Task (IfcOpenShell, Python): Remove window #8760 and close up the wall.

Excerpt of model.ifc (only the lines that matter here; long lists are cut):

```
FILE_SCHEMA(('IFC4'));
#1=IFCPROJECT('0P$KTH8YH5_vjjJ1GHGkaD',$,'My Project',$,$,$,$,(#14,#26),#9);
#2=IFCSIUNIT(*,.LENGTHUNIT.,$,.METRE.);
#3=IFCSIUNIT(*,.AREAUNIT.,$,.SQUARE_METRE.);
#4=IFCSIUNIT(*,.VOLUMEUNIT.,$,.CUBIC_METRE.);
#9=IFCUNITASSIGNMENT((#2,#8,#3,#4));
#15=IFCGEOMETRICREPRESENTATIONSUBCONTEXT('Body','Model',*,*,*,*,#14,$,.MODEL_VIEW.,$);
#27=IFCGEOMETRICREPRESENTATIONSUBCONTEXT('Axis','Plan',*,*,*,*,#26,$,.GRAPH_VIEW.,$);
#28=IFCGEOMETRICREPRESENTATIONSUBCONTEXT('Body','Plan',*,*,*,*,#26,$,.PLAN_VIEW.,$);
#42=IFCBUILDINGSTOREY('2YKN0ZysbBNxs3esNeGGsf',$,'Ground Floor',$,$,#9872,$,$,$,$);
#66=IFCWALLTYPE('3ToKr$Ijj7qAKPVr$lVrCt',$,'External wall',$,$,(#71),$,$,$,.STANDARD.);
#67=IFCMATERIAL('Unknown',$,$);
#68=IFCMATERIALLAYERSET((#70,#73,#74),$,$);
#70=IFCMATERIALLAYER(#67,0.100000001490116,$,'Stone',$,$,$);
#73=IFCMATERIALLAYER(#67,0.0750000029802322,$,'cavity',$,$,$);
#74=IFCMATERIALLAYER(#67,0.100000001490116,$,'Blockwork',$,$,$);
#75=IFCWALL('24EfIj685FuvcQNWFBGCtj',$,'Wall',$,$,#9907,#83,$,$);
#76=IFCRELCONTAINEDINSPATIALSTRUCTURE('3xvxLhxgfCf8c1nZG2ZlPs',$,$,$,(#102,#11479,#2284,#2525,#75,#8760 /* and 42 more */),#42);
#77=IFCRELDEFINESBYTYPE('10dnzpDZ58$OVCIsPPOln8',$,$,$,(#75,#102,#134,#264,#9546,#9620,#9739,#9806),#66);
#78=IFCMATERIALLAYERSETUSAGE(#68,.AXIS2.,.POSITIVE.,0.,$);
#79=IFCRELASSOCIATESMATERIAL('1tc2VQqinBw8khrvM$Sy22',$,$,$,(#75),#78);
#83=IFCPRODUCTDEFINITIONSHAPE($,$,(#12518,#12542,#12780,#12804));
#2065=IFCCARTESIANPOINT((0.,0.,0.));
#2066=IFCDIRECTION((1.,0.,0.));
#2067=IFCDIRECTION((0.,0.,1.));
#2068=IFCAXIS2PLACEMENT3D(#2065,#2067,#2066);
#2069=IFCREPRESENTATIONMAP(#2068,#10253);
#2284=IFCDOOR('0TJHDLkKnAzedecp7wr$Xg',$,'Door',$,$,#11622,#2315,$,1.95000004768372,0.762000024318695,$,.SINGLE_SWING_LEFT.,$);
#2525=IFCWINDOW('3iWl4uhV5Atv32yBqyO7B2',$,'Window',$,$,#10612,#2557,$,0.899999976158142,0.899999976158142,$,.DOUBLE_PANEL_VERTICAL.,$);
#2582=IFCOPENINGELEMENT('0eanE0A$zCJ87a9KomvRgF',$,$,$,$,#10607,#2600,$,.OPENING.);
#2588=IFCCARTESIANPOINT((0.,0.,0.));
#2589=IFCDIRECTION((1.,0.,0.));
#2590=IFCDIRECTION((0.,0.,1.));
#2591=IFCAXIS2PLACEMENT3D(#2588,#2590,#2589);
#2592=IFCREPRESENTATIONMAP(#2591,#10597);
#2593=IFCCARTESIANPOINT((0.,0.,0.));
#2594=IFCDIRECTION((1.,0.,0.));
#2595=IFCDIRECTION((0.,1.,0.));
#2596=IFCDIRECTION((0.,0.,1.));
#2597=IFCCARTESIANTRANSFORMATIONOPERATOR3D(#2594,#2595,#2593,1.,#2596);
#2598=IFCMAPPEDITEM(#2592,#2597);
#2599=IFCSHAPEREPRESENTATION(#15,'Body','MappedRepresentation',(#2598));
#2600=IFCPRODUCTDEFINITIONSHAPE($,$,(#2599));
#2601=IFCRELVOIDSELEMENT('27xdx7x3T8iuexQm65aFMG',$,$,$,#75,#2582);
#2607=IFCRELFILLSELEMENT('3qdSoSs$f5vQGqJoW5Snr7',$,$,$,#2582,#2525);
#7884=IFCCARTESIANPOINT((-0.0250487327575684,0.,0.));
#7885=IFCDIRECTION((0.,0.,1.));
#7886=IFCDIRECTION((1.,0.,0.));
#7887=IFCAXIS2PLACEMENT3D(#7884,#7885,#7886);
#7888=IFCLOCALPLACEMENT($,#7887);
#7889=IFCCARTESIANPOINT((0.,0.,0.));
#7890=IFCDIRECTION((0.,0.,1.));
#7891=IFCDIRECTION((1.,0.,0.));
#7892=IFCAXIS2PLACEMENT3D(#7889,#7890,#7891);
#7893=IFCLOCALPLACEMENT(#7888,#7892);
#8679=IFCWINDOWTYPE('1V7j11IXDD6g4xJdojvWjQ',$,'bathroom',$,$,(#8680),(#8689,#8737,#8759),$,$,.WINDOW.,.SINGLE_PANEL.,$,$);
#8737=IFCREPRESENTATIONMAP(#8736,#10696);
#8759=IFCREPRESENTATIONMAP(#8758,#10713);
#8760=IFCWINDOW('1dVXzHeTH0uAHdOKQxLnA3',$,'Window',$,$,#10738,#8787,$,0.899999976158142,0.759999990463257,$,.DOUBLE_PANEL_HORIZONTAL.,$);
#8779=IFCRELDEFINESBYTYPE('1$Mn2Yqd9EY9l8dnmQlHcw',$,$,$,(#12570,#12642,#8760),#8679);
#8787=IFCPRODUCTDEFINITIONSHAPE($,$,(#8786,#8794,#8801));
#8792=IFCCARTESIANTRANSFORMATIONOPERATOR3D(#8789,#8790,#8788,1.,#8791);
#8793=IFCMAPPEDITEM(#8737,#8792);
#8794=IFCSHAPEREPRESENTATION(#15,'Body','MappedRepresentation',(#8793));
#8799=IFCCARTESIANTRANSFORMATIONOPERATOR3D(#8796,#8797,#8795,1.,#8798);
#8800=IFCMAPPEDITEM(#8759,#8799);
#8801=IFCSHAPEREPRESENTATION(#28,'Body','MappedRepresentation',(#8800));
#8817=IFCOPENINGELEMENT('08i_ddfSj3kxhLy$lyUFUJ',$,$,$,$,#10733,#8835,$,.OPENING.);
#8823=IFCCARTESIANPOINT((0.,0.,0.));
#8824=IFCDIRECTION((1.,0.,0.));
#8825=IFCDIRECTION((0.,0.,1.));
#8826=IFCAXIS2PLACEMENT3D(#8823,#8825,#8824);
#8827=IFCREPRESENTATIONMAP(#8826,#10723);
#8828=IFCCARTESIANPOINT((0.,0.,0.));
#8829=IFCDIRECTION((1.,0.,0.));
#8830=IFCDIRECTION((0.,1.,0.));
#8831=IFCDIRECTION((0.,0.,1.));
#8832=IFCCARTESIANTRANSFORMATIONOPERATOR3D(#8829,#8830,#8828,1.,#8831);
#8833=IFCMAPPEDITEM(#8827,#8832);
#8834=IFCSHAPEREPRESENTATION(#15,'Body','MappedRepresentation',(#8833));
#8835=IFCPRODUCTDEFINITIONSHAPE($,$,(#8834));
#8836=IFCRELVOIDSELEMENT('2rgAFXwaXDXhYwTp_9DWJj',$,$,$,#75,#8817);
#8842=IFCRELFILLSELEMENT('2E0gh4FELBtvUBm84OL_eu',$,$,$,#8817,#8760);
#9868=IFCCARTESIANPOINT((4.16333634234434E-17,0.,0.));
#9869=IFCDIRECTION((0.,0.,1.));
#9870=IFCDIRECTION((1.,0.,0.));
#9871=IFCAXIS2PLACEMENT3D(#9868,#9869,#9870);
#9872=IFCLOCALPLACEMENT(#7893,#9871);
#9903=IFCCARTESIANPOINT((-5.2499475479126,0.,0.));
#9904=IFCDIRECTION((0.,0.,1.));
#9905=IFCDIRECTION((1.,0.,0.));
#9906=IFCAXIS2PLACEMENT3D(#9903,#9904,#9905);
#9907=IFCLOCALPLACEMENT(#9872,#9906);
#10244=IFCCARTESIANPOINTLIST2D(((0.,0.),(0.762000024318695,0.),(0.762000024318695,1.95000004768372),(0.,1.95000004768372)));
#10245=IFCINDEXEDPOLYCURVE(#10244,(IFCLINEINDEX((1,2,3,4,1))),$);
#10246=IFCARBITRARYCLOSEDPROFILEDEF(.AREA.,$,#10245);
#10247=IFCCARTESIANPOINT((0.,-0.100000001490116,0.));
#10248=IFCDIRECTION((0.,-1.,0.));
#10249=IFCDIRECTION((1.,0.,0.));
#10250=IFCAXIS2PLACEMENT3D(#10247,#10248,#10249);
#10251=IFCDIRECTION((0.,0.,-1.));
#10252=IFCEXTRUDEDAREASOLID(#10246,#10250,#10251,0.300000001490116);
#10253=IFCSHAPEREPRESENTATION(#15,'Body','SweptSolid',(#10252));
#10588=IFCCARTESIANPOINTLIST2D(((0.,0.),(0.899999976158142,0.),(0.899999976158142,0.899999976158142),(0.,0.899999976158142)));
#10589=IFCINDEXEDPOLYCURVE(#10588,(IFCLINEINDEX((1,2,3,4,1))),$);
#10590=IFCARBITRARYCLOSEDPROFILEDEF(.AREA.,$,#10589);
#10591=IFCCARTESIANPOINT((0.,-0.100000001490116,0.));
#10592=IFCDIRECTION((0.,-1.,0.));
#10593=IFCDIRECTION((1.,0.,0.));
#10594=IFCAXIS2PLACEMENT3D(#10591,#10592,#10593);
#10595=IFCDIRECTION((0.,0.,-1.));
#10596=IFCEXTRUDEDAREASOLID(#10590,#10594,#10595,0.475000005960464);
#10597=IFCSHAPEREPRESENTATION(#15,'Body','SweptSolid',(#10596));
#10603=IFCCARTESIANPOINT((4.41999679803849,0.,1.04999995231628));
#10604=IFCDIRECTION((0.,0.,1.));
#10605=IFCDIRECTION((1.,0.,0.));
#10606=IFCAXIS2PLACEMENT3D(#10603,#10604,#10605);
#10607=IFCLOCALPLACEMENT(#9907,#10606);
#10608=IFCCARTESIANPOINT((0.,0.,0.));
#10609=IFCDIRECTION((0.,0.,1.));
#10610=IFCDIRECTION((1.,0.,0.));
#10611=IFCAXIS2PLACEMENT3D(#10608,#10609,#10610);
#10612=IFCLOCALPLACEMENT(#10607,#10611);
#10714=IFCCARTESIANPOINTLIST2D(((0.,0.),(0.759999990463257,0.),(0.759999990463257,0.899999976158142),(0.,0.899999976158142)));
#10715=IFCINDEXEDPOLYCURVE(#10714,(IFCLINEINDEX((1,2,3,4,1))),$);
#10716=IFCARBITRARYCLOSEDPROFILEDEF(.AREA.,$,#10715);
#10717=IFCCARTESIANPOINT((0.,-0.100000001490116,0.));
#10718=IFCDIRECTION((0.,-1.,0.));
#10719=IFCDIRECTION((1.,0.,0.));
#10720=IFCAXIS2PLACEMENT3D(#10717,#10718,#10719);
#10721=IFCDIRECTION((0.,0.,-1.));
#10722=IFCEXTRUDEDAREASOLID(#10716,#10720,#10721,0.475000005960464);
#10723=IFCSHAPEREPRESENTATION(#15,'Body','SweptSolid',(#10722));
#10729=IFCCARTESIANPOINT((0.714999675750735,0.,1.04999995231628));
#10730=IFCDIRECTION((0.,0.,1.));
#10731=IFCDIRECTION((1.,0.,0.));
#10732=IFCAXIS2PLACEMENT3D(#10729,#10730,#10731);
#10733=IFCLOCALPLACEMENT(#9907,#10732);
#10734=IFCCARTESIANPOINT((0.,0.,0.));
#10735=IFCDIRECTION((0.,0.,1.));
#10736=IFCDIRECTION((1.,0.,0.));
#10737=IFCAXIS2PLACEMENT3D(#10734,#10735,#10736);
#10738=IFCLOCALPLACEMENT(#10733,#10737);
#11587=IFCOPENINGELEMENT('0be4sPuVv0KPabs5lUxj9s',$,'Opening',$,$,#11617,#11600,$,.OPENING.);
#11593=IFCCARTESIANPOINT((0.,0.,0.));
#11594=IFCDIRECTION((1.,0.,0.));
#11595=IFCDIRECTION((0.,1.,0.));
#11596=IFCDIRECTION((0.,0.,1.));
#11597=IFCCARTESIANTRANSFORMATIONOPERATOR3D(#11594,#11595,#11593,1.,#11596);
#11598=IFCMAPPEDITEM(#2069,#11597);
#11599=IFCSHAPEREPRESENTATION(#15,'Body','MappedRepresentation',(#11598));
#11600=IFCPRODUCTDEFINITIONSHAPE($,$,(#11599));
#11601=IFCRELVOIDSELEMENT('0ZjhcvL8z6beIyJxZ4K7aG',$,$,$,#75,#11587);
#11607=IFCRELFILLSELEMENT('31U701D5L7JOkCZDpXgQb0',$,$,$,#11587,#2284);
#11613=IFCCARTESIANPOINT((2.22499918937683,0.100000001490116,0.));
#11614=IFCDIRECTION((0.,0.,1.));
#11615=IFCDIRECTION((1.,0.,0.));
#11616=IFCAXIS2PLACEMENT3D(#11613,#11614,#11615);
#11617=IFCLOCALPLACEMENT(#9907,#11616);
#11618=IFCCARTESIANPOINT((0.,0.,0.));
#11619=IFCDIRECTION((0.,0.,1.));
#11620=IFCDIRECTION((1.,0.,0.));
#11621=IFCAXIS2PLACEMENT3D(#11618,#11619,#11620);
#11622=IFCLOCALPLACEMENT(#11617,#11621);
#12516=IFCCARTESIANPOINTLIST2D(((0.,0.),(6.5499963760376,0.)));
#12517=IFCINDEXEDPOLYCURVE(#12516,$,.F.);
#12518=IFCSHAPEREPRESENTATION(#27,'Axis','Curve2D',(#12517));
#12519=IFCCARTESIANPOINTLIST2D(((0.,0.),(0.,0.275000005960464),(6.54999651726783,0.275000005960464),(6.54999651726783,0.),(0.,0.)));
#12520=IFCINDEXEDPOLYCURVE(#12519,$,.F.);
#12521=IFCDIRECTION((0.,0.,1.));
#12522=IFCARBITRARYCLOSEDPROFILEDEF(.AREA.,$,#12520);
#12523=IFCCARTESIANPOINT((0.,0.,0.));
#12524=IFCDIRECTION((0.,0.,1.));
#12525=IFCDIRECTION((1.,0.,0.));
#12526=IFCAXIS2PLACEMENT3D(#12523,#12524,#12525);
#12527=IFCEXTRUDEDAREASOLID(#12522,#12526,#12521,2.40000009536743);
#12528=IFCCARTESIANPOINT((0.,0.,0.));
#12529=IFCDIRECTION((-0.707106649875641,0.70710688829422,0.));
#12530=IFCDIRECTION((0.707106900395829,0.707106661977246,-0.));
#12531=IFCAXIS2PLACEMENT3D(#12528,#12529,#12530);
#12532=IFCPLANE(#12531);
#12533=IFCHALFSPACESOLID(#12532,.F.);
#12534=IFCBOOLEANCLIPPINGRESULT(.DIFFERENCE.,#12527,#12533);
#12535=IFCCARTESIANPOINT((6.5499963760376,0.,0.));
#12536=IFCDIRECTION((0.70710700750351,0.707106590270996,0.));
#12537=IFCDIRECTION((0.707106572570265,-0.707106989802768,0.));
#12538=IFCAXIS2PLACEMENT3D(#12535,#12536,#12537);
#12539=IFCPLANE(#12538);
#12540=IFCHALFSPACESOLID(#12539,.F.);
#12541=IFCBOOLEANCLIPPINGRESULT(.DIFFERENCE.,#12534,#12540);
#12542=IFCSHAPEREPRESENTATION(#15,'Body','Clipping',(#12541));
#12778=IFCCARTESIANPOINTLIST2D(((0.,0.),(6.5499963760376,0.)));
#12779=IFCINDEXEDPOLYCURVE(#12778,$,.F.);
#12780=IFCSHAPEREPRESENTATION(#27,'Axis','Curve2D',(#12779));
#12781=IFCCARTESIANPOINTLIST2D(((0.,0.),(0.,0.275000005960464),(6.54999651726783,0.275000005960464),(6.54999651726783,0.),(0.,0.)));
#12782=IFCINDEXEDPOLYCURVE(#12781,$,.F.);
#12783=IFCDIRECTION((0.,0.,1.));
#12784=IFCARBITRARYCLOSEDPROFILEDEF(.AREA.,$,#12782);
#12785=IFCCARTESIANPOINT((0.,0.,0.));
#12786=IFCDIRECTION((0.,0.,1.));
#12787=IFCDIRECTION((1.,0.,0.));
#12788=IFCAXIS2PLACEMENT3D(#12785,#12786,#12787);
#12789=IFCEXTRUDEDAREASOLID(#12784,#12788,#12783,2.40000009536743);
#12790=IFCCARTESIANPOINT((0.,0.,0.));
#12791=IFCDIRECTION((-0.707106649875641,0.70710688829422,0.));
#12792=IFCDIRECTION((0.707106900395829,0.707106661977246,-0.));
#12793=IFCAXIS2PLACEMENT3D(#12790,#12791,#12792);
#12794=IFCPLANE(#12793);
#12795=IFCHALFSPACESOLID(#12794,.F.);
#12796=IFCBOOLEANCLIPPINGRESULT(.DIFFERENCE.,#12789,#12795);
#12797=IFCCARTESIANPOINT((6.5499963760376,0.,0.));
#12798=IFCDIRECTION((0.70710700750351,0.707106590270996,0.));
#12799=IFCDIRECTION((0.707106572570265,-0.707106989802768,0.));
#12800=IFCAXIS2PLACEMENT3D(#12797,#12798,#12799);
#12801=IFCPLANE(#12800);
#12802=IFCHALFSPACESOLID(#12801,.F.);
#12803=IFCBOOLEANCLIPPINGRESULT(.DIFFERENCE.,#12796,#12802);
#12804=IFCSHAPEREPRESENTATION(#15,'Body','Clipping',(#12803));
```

```python
import ifcopenshell
import ifcopenshell.api.feature
import ifcopenshell.api.root
import ifcopenshell.geom
import ifcopenshell.util.shape

model = ifcopenshell.open("model.ifc")
settings = ifcopenshell.geom.settings()


def volume(element):
    """Net volume in cubic metres, openings subtracted."""
    shape = ifcopenshell.geom.create_shape(settings, element)
    return ifcopenshell.util.shape.get_volume(shape.geometry)


window = model.by_id(8760)
opening = window.FillsVoids[0].RelatingOpeningElement
wall = opening.VoidsElements[0].RelatingBuildingElement
before = volume(wall)

ifcopenshell.api.root.remove_product(model, product=window)
ifcopenshell.api.feature.remove_feature(model, feature=opening)

after = volume(wall)

print(f"wall volume {before:.3f} -> {after:.3f} m3")

model.write("model_v2.ifc")
```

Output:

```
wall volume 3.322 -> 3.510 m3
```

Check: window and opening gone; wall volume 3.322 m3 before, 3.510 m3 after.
